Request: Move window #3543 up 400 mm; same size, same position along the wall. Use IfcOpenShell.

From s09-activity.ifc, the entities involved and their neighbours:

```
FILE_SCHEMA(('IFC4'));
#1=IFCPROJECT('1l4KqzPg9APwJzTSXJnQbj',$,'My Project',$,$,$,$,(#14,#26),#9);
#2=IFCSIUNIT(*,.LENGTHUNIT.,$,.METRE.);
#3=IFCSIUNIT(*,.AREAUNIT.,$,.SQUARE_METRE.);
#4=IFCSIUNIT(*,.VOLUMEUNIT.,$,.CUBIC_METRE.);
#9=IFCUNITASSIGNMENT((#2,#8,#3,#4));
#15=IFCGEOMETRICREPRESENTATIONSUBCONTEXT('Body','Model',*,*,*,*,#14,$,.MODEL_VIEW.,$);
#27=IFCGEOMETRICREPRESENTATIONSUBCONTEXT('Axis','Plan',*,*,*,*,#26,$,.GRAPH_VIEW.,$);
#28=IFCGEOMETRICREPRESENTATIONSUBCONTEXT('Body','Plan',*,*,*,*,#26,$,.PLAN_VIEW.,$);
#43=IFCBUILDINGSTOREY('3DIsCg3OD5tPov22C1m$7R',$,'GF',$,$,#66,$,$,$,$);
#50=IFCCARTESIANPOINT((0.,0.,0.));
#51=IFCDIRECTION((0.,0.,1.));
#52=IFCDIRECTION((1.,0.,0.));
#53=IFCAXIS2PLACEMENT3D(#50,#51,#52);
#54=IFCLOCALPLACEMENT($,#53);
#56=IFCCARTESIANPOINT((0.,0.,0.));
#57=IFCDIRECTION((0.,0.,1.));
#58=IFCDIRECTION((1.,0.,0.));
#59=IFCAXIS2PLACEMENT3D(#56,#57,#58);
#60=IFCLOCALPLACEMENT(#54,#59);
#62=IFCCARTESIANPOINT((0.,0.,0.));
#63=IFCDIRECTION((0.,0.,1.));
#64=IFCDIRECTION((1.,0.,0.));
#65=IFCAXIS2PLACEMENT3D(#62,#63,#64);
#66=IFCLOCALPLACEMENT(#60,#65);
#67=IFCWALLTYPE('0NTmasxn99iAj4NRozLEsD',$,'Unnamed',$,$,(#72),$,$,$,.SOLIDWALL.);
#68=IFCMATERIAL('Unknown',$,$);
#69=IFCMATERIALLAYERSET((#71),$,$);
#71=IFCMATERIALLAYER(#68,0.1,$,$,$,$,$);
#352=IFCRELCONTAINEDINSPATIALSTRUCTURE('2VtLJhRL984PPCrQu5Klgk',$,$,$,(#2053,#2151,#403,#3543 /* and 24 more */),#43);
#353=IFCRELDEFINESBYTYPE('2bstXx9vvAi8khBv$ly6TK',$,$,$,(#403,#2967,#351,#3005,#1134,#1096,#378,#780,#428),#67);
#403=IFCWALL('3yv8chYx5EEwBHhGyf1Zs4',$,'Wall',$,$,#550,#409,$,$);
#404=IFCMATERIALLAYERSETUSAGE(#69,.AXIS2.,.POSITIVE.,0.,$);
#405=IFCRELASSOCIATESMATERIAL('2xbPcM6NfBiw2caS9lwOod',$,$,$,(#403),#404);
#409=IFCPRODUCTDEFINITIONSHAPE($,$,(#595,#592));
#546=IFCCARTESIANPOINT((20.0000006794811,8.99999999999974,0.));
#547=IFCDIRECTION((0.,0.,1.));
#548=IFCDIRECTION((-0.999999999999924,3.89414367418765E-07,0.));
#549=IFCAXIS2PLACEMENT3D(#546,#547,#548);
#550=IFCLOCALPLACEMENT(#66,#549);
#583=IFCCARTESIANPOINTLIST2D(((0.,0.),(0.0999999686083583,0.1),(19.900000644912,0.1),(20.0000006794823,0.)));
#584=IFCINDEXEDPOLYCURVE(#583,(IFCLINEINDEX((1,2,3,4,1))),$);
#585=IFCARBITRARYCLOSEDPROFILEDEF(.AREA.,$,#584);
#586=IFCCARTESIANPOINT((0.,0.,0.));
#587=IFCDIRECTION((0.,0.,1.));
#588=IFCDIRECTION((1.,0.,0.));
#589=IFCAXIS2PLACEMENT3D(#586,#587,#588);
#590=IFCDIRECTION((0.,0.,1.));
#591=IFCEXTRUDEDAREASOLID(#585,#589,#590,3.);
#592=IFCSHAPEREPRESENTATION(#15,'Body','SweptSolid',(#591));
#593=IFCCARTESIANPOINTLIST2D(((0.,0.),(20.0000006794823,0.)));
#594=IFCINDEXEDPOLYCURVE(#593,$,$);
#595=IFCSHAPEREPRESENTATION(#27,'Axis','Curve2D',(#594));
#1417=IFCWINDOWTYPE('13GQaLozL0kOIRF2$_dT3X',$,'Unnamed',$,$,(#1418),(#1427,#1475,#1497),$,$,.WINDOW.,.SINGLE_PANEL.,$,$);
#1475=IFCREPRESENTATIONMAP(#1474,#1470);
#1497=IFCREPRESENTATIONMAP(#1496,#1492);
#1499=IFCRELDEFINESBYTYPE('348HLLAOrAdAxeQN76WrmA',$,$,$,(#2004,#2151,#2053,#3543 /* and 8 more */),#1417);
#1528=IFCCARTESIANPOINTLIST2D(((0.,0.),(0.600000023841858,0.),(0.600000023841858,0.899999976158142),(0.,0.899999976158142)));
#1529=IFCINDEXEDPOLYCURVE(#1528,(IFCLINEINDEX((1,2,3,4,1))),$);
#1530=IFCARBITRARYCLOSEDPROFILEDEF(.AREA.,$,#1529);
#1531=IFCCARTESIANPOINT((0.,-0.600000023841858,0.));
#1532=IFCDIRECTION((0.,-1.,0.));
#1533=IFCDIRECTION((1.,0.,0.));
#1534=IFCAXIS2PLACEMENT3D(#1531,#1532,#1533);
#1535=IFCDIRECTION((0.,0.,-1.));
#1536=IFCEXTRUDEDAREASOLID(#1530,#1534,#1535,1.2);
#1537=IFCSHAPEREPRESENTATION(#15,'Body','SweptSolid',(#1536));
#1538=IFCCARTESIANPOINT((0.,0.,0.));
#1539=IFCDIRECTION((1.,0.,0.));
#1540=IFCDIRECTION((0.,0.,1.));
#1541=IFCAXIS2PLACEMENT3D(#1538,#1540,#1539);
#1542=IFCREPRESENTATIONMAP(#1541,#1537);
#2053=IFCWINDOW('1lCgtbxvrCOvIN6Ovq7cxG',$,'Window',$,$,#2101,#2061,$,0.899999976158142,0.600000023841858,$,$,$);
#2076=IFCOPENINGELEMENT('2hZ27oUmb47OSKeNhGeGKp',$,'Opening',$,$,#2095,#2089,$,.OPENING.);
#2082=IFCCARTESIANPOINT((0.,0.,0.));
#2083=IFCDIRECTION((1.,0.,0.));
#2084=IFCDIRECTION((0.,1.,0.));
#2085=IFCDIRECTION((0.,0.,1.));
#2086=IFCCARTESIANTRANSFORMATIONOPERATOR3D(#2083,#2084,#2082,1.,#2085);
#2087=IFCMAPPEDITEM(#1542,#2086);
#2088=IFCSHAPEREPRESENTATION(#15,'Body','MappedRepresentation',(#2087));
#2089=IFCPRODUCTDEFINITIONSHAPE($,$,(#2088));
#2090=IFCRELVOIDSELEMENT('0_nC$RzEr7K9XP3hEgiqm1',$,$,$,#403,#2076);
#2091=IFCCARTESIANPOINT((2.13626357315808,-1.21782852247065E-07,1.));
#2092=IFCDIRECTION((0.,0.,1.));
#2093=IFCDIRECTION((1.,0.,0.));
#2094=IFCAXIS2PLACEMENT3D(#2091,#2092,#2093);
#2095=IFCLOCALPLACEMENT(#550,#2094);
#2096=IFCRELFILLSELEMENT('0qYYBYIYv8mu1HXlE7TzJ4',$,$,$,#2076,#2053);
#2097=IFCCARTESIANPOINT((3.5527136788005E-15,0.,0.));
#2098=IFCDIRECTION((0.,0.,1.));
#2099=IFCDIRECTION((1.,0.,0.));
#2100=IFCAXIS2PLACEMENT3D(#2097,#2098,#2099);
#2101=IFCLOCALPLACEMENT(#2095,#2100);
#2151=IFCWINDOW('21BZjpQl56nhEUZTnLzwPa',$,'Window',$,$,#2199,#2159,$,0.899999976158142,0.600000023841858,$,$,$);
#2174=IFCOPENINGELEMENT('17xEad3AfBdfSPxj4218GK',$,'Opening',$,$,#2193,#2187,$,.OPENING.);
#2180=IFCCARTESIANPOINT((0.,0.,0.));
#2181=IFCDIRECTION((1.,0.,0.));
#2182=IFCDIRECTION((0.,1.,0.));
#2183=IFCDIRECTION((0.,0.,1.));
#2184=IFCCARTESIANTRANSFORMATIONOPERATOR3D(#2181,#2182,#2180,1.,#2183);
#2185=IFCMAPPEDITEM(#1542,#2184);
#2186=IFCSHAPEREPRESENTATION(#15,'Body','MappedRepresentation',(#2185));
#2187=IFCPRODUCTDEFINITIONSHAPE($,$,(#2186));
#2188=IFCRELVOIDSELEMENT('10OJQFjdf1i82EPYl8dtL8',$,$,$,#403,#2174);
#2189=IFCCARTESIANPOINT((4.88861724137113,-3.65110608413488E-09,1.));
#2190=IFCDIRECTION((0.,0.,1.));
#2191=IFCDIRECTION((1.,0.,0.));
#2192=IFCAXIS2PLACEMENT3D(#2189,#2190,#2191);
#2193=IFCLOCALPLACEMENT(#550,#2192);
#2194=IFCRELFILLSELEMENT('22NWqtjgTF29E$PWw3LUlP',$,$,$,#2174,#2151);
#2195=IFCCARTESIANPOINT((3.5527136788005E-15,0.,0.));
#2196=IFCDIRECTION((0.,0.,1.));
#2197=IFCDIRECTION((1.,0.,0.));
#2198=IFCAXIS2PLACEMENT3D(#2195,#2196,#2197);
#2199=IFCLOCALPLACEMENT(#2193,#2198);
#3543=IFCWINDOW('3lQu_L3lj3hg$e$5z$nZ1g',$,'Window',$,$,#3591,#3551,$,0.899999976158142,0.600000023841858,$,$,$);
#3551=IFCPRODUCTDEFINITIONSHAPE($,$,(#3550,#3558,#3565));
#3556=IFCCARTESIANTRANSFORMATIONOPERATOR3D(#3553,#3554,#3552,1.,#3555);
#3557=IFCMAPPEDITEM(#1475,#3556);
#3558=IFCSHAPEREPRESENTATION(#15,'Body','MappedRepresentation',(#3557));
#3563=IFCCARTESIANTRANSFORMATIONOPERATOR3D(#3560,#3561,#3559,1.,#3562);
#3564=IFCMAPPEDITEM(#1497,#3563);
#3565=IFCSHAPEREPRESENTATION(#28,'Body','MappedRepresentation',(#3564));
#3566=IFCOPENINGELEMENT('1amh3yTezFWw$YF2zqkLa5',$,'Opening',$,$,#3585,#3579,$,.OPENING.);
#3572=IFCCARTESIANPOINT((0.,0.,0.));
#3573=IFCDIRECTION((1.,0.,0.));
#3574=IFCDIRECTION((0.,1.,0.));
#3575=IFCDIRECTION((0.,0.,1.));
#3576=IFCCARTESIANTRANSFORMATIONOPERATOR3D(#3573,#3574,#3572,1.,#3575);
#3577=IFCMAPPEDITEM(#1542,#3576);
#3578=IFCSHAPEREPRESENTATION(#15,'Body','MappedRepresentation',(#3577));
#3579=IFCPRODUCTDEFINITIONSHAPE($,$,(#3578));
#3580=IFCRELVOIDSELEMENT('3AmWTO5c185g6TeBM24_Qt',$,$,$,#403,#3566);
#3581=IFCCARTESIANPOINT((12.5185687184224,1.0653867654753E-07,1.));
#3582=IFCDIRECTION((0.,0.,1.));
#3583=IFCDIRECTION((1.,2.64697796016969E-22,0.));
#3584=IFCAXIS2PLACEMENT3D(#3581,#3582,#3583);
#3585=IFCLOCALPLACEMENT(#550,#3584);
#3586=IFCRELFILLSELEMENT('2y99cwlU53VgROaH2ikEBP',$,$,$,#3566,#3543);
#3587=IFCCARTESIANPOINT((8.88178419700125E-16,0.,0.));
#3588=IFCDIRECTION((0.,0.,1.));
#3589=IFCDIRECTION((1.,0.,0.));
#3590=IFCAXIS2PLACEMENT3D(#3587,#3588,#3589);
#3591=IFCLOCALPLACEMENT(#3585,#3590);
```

```python
import numpy as np
import ifcopenshell
import ifcopenshell.api.geometry
import ifcopenshell.util.placement
import ifcopenshell.util.unit

model = ifcopenshell.open("s09-activity.ifc")
unit_scale = ifcopenshell.util.unit.calculate_unit_scale(model)

window = model.by_guid("3lQu_L3lj3hg$e$5z$nZ1g")
opening = window.FillsVoids[0].RelatingOpeningElement
dz = 0.4

shift = np.array([0.0, 0.0, dz])
# The window is placed relative to its opening, so it follows when the opening moves.
matrix = ifcopenshell.util.placement.get_local_placement(opening.ObjectPlacement)
matrix[:3, 3] += shift
ifcopenshell.api.geometry.edit_object_placement(
    model, product=opening, matrix=matrix, is_si=False, should_transform_children=True
)

print(f"moved by {dz * unit_scale:+.3f} m")

model.write("s09-activity_edited.ifc")
```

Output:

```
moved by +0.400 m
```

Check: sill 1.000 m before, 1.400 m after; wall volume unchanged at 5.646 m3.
